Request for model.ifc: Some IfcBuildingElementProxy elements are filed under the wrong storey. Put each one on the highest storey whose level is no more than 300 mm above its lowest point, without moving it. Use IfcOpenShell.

First a look at what the model holds.

```python
import ifcopenshell
import ifcopenshell.util.element
import ifcopenshell.util.placement

model = ifcopenshell.open("model.ifc")
print(model.schema)
for storey in model.by_type("IfcBuildingStorey"):
    level = ifcopenshell.util.placement.get_storey_elevation(storey)
    count = sum(e.is_a("IfcBuildingElementProxy") for e in ifcopenshell.util.element.get_contained(storey))
    print(storey.id(), storey.Name, round(level, 3), count, sep=" | ")
```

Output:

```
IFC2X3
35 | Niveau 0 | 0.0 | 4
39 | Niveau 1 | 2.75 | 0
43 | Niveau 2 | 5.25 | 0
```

```python
import ifcopenshell
import ifcopenshell.api.spatial
import ifcopenshell.geom
import ifcopenshell.util.element
import ifcopenshell.util.placement
import ifcopenshell.util.shape
import ifcopenshell.util.unit

model = ifcopenshell.open("model.ifc")
unit_scale = ifcopenshell.util.unit.calculate_unit_scale(model)
settings = ifcopenshell.geom.settings()

levels = sorted(
    ((ifcopenshell.util.placement.get_storey_elevation(s) * unit_scale, s) for s in model.by_type("IfcBuildingStorey")),
    key=lambda pair: pair[0],
)

for e in model.by_type("IfcBuildingElementProxy"):
    current = e.ContainedInStructure[0].RelatingStructure if e.ContainedInStructure else None
    if current is None or not current.is_a("IfcBuildingStorey"):
        continue
    shape = ifcopenshell.geom.create_shape(settings, e)
    bottom = ifcopenshell.util.shape.get_shape_bottom_elevation(shape, shape.geometry)
    below = [s for level, s in levels if level <= bottom + 0.3]
    storey = below[-1] if below else levels[0][1]
    if storey != current:
        # assign_container keeps the world position.
        ifcopenshell.api.spatial.assign_container(model, products=[e], relating_structure=storey)
        print(e.id(), current.Name, "->", storey.Name)

model.write("model_edited.ifc")
```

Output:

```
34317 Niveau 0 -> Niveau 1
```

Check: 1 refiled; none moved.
